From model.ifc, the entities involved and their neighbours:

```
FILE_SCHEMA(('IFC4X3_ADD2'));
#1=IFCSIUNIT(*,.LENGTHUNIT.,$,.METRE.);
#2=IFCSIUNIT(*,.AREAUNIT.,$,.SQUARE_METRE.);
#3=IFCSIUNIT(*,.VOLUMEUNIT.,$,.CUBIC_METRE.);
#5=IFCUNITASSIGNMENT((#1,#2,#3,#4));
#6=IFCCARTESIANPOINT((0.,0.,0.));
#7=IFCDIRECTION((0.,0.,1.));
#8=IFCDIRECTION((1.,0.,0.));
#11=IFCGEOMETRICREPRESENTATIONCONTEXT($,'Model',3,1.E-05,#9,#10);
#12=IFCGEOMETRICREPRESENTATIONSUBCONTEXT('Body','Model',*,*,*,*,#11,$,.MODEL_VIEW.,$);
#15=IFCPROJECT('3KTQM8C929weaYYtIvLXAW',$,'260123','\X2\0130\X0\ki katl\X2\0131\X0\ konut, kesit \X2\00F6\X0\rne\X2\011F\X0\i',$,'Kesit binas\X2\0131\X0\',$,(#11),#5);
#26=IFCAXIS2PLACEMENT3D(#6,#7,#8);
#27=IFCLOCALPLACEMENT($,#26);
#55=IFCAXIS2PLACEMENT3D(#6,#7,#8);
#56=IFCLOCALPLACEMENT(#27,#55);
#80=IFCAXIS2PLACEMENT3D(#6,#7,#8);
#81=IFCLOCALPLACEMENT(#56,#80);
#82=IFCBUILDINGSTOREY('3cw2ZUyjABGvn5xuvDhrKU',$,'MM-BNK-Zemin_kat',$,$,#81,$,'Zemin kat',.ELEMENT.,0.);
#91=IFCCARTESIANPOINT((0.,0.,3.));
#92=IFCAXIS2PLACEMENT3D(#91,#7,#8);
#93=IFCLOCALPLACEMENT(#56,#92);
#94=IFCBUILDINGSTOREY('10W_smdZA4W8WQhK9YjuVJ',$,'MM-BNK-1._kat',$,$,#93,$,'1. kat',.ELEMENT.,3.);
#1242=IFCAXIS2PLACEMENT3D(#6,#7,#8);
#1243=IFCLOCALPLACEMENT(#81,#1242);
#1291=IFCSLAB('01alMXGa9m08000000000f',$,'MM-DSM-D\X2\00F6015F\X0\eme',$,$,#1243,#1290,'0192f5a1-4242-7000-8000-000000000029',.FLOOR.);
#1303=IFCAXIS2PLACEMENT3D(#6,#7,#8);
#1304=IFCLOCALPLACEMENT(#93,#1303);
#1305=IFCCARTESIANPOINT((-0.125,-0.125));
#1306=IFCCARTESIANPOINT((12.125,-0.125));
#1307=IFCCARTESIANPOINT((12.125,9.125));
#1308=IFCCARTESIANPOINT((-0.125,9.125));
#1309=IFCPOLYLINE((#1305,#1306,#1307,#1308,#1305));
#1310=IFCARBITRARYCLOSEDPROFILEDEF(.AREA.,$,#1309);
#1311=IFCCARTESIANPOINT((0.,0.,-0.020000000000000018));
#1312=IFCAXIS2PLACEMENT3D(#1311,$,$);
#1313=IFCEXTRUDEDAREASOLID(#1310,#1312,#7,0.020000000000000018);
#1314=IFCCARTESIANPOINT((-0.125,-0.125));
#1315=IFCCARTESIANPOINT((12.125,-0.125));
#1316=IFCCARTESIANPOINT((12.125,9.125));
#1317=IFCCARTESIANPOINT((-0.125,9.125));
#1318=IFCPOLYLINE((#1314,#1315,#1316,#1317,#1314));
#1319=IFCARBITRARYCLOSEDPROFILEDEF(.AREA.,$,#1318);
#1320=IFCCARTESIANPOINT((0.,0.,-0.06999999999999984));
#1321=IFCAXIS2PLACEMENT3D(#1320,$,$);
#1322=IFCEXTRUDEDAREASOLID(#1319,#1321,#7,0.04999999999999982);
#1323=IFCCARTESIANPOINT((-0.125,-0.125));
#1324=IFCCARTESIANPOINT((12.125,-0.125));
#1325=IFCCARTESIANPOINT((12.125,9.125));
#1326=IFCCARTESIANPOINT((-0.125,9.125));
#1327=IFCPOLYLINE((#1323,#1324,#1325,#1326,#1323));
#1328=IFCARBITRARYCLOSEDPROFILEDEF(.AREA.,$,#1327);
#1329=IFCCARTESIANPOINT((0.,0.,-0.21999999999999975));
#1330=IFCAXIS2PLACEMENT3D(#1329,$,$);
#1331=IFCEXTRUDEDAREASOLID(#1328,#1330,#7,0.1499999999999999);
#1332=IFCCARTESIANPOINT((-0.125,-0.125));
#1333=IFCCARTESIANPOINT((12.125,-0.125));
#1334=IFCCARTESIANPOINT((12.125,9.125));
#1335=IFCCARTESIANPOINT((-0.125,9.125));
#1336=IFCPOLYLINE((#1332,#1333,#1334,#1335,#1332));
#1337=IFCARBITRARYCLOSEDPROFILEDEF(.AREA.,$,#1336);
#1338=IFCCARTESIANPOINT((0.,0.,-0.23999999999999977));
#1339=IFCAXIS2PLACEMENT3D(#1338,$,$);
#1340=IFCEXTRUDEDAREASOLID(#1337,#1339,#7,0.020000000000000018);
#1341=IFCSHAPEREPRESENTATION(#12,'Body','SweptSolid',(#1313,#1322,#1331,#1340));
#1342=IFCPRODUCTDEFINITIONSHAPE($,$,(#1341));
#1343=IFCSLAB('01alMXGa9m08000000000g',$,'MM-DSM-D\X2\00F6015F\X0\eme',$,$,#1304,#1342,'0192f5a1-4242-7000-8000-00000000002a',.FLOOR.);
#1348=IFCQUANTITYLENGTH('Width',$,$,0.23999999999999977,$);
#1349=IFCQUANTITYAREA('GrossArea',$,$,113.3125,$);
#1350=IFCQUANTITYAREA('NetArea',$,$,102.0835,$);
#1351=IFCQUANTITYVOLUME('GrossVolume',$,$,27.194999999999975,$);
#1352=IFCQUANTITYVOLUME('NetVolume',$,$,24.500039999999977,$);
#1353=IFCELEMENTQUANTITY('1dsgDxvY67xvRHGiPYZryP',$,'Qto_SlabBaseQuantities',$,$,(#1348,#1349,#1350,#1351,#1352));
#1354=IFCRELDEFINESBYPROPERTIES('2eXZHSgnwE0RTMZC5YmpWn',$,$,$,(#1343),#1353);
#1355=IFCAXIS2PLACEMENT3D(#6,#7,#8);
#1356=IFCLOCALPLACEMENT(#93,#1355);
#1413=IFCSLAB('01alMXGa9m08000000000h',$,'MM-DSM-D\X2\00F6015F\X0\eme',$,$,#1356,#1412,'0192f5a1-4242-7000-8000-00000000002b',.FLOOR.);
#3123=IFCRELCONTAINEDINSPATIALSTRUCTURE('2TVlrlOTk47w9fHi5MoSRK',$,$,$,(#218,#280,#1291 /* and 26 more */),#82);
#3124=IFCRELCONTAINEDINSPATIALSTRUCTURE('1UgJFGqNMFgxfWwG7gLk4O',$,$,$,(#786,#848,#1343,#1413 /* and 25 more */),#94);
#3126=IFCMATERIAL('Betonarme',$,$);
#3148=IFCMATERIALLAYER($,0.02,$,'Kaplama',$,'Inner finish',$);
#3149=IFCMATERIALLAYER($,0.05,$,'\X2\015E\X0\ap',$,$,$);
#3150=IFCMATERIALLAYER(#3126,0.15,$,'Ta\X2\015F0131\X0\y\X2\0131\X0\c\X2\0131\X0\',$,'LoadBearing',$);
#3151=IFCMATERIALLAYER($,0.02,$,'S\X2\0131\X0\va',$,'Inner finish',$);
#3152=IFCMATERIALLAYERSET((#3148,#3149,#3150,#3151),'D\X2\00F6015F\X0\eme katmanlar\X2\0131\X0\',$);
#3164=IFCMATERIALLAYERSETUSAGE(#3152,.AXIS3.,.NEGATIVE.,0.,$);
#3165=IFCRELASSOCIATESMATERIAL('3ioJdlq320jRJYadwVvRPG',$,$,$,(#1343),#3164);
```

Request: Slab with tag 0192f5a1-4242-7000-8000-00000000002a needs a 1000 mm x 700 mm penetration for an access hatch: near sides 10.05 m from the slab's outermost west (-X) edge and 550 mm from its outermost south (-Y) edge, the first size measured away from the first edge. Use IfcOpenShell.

```python
import numpy as np
import ifcopenshell
import ifcopenshell.api.feature
import ifcopenshell.api.geometry
import ifcopenshell.api.pset
import ifcopenshell.api.root
import ifcopenshell.geom
import ifcopenshell.util.element
import ifcopenshell.util.placement
import ifcopenshell.util.representation
import ifcopenshell.util.shape
import ifcopenshell.util.unit

model = ifcopenshell.open("model.ifc")
unit_scale = ifcopenshell.util.unit.calculate_unit_scale(model)
area_scale = ifcopenshell.util.unit.calculate_unit_scale(model, "AREAUNIT")
volume_scale = ifcopenshell.util.unit.calculate_unit_scale(model, "VOLUMEUNIT")
settings = ifcopenshell.geom.settings()


def volume(element):
    """Net volume in cubic metres, openings subtracted."""
    shape = ifcopenshell.geom.create_shape(settings, element)
    return ifcopenshell.util.shape.get_volume(shape.geometry)


slab = model.by_guid("01alMXGa9m08000000000g")
before = volume(slab)

# Extent in the slab's own axes, in metres. The edges named are its -X and -Y sides.
slab_shape = ifcopenshell.geom.create_shape(settings, slab)
vertices = ifcopenshell.util.shape.get_vertices(slab_shape.geometry)
x_min, y_min, bottom = vertices.min(axis=0)
top = vertices[:, 2].max()

opening = ifcopenshell.api.root.create_entity(model, ifc_class="IfcOpeningElement", name="Access hatch opening", predefined_type="OPENING")
context = ifcopenshell.util.representation.get_context(model, "Model", "Body", "MODEL_VIEW")
width, depth = 1, 0.7
outline = [(0.0, 0.0), (width, 0.0), (width, depth), (0.0, depth), (0.0, 0.0)]
# Overshoot both faces by 50 mm so the cut is clean.
shape = ifcopenshell.api.geometry.add_slab_representation(
    model, context=context, depth=top - bottom + 0.1, polyline=outline
)
ifcopenshell.api.geometry.assign_representation(model, product=opening, representation=shape)

matrix = ifcopenshell.util.placement.get_local_placement(slab.ObjectPlacement)
matrix[:, 3] = matrix @ np.append(np.array([x_min + 10.05, y_min + 0.55, bottom - 0.05]) / unit_scale, 1.0)
ifcopenshell.api.geometry.edit_object_placement(model, product=opening, matrix=matrix, is_si=False)
ifcopenshell.api.feature.add_feature(model, feature=opening, element=slab)

after = volume(slab)

# Update the slab's stored quantities.
qto = model.by_id(ifcopenshell.util.element.get_pset(slab, "Qto_SlabBaseQuantities", should_inherit=False)["id"])
ifcopenshell.api.pset.edit_qto(model, qto=qto, properties={
    "NetArea": after / (top - bottom) / area_scale,
    "NetVolume": after / volume_scale,
})

print(f"slab volume {before:.3f} -> {after:.3f} m3")

model.write("model-out.ifc")
```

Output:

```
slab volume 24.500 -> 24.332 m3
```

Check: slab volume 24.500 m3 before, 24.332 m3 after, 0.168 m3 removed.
